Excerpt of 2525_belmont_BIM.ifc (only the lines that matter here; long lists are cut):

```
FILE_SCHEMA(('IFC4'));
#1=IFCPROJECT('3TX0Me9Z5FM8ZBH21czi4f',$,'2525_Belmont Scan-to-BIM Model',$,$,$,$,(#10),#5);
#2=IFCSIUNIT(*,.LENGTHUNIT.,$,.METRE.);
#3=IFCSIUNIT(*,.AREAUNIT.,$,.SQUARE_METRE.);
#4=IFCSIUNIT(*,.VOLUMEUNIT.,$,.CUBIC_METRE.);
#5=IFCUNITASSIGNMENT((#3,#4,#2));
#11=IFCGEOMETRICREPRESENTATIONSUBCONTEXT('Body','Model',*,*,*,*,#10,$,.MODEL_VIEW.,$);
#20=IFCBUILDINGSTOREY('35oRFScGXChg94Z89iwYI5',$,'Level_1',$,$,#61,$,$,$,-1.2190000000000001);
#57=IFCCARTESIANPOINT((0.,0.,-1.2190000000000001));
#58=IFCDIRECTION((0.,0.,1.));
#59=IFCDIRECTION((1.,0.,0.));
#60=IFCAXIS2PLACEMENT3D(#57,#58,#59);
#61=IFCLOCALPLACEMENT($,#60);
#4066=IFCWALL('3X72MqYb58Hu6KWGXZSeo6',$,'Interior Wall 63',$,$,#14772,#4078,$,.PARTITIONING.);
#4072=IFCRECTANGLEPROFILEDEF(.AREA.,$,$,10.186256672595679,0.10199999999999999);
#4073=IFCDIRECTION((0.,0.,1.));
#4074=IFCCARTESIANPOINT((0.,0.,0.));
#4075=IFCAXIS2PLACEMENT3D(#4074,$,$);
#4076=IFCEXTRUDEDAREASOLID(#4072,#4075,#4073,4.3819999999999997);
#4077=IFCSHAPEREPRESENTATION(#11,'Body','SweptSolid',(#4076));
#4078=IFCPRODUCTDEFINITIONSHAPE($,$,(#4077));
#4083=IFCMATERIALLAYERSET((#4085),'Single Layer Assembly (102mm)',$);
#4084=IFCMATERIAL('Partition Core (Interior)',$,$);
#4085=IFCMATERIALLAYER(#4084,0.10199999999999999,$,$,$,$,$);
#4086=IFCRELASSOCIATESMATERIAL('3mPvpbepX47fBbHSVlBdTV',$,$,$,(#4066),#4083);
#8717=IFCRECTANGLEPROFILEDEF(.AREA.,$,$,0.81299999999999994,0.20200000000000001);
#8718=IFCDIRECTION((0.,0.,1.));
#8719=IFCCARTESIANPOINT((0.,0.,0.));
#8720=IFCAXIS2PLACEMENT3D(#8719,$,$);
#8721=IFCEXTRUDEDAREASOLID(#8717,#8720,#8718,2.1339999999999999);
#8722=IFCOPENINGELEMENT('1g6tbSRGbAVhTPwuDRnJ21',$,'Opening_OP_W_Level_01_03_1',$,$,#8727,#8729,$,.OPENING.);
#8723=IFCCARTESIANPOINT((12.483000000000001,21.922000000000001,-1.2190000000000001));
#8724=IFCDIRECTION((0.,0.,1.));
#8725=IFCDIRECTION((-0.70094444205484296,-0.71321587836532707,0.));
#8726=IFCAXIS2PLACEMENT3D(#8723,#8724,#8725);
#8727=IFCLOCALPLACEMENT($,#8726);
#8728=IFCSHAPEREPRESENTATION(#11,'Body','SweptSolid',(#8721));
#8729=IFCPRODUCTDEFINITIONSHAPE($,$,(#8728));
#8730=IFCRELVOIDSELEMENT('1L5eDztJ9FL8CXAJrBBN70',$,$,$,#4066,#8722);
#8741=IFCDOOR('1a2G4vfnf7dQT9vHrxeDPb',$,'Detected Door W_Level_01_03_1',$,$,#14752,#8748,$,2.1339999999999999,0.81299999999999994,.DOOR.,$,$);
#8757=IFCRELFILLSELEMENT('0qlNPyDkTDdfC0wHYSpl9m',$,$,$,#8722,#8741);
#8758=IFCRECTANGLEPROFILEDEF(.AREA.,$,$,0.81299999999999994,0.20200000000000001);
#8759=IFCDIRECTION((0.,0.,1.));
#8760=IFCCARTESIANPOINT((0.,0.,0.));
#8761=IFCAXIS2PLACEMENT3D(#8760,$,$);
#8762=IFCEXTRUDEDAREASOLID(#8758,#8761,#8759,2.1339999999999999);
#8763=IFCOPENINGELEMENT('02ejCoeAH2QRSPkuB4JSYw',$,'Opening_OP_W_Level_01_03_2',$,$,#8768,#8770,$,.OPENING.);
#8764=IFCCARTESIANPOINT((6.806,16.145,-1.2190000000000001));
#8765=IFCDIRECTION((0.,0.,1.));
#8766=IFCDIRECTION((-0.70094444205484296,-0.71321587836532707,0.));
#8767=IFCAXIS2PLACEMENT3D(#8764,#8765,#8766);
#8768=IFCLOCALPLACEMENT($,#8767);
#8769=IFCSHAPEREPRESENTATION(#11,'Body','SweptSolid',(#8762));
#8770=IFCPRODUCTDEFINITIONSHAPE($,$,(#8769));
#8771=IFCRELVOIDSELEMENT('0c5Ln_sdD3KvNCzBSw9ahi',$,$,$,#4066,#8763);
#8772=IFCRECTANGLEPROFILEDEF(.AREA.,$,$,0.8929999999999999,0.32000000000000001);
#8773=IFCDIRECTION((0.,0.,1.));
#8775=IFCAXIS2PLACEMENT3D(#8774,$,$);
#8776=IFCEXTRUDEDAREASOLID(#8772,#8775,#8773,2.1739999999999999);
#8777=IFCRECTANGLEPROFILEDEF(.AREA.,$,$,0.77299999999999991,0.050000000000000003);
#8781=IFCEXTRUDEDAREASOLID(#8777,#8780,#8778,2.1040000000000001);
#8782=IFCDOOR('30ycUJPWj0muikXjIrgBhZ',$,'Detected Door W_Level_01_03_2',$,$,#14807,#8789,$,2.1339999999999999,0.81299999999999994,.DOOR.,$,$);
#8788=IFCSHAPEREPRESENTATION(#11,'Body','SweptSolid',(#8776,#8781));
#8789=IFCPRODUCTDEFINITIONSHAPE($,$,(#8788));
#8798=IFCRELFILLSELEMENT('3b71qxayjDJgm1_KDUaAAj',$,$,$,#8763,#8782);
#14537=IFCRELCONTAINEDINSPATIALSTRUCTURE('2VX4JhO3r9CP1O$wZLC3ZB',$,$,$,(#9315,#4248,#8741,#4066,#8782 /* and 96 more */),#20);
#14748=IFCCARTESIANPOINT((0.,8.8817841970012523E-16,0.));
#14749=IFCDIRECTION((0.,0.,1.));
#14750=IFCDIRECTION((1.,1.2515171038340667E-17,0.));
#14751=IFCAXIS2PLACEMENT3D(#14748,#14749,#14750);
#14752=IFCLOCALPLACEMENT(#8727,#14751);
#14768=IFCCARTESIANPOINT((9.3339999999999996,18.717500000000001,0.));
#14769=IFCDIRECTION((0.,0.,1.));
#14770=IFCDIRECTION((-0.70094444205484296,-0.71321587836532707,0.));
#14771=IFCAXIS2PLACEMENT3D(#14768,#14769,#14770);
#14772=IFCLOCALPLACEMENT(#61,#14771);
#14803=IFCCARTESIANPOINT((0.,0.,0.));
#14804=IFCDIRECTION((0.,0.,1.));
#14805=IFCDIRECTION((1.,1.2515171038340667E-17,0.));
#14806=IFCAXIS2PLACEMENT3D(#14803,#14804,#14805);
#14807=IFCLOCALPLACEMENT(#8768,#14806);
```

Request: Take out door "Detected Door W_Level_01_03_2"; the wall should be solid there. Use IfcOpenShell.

```python
import ifcopenshell
import ifcopenshell.api.feature
import ifcopenshell.api.root
import ifcopenshell.geom
import ifcopenshell.util.shape

model = ifcopenshell.open("2525_belmont_BIM.ifc")
settings = ifcopenshell.geom.settings()


def volume(element):
    """Net volume in cubic metres, openings subtracted."""
    shape = ifcopenshell.geom.create_shape(settings, element)
    return ifcopenshell.util.shape.get_volume(shape.geometry)


door = model.by_id(8782)
opening = door.FillsVoids[0].RelatingOpeningElement
wall = opening.VoidsElements[0].RelatingBuildingElement
before = volume(wall)

ifcopenshell.api.root.remove_product(model, product=door)
ifcopenshell.api.feature.remove_feature(model, feature=opening)

after = volume(wall)

print(f"wall volume {before:.3f} -> {after:.3f} m3")

model.write("2525_belmont_BIM_v2.ifc")
```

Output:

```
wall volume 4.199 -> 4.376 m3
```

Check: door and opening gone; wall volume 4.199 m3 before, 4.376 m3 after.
